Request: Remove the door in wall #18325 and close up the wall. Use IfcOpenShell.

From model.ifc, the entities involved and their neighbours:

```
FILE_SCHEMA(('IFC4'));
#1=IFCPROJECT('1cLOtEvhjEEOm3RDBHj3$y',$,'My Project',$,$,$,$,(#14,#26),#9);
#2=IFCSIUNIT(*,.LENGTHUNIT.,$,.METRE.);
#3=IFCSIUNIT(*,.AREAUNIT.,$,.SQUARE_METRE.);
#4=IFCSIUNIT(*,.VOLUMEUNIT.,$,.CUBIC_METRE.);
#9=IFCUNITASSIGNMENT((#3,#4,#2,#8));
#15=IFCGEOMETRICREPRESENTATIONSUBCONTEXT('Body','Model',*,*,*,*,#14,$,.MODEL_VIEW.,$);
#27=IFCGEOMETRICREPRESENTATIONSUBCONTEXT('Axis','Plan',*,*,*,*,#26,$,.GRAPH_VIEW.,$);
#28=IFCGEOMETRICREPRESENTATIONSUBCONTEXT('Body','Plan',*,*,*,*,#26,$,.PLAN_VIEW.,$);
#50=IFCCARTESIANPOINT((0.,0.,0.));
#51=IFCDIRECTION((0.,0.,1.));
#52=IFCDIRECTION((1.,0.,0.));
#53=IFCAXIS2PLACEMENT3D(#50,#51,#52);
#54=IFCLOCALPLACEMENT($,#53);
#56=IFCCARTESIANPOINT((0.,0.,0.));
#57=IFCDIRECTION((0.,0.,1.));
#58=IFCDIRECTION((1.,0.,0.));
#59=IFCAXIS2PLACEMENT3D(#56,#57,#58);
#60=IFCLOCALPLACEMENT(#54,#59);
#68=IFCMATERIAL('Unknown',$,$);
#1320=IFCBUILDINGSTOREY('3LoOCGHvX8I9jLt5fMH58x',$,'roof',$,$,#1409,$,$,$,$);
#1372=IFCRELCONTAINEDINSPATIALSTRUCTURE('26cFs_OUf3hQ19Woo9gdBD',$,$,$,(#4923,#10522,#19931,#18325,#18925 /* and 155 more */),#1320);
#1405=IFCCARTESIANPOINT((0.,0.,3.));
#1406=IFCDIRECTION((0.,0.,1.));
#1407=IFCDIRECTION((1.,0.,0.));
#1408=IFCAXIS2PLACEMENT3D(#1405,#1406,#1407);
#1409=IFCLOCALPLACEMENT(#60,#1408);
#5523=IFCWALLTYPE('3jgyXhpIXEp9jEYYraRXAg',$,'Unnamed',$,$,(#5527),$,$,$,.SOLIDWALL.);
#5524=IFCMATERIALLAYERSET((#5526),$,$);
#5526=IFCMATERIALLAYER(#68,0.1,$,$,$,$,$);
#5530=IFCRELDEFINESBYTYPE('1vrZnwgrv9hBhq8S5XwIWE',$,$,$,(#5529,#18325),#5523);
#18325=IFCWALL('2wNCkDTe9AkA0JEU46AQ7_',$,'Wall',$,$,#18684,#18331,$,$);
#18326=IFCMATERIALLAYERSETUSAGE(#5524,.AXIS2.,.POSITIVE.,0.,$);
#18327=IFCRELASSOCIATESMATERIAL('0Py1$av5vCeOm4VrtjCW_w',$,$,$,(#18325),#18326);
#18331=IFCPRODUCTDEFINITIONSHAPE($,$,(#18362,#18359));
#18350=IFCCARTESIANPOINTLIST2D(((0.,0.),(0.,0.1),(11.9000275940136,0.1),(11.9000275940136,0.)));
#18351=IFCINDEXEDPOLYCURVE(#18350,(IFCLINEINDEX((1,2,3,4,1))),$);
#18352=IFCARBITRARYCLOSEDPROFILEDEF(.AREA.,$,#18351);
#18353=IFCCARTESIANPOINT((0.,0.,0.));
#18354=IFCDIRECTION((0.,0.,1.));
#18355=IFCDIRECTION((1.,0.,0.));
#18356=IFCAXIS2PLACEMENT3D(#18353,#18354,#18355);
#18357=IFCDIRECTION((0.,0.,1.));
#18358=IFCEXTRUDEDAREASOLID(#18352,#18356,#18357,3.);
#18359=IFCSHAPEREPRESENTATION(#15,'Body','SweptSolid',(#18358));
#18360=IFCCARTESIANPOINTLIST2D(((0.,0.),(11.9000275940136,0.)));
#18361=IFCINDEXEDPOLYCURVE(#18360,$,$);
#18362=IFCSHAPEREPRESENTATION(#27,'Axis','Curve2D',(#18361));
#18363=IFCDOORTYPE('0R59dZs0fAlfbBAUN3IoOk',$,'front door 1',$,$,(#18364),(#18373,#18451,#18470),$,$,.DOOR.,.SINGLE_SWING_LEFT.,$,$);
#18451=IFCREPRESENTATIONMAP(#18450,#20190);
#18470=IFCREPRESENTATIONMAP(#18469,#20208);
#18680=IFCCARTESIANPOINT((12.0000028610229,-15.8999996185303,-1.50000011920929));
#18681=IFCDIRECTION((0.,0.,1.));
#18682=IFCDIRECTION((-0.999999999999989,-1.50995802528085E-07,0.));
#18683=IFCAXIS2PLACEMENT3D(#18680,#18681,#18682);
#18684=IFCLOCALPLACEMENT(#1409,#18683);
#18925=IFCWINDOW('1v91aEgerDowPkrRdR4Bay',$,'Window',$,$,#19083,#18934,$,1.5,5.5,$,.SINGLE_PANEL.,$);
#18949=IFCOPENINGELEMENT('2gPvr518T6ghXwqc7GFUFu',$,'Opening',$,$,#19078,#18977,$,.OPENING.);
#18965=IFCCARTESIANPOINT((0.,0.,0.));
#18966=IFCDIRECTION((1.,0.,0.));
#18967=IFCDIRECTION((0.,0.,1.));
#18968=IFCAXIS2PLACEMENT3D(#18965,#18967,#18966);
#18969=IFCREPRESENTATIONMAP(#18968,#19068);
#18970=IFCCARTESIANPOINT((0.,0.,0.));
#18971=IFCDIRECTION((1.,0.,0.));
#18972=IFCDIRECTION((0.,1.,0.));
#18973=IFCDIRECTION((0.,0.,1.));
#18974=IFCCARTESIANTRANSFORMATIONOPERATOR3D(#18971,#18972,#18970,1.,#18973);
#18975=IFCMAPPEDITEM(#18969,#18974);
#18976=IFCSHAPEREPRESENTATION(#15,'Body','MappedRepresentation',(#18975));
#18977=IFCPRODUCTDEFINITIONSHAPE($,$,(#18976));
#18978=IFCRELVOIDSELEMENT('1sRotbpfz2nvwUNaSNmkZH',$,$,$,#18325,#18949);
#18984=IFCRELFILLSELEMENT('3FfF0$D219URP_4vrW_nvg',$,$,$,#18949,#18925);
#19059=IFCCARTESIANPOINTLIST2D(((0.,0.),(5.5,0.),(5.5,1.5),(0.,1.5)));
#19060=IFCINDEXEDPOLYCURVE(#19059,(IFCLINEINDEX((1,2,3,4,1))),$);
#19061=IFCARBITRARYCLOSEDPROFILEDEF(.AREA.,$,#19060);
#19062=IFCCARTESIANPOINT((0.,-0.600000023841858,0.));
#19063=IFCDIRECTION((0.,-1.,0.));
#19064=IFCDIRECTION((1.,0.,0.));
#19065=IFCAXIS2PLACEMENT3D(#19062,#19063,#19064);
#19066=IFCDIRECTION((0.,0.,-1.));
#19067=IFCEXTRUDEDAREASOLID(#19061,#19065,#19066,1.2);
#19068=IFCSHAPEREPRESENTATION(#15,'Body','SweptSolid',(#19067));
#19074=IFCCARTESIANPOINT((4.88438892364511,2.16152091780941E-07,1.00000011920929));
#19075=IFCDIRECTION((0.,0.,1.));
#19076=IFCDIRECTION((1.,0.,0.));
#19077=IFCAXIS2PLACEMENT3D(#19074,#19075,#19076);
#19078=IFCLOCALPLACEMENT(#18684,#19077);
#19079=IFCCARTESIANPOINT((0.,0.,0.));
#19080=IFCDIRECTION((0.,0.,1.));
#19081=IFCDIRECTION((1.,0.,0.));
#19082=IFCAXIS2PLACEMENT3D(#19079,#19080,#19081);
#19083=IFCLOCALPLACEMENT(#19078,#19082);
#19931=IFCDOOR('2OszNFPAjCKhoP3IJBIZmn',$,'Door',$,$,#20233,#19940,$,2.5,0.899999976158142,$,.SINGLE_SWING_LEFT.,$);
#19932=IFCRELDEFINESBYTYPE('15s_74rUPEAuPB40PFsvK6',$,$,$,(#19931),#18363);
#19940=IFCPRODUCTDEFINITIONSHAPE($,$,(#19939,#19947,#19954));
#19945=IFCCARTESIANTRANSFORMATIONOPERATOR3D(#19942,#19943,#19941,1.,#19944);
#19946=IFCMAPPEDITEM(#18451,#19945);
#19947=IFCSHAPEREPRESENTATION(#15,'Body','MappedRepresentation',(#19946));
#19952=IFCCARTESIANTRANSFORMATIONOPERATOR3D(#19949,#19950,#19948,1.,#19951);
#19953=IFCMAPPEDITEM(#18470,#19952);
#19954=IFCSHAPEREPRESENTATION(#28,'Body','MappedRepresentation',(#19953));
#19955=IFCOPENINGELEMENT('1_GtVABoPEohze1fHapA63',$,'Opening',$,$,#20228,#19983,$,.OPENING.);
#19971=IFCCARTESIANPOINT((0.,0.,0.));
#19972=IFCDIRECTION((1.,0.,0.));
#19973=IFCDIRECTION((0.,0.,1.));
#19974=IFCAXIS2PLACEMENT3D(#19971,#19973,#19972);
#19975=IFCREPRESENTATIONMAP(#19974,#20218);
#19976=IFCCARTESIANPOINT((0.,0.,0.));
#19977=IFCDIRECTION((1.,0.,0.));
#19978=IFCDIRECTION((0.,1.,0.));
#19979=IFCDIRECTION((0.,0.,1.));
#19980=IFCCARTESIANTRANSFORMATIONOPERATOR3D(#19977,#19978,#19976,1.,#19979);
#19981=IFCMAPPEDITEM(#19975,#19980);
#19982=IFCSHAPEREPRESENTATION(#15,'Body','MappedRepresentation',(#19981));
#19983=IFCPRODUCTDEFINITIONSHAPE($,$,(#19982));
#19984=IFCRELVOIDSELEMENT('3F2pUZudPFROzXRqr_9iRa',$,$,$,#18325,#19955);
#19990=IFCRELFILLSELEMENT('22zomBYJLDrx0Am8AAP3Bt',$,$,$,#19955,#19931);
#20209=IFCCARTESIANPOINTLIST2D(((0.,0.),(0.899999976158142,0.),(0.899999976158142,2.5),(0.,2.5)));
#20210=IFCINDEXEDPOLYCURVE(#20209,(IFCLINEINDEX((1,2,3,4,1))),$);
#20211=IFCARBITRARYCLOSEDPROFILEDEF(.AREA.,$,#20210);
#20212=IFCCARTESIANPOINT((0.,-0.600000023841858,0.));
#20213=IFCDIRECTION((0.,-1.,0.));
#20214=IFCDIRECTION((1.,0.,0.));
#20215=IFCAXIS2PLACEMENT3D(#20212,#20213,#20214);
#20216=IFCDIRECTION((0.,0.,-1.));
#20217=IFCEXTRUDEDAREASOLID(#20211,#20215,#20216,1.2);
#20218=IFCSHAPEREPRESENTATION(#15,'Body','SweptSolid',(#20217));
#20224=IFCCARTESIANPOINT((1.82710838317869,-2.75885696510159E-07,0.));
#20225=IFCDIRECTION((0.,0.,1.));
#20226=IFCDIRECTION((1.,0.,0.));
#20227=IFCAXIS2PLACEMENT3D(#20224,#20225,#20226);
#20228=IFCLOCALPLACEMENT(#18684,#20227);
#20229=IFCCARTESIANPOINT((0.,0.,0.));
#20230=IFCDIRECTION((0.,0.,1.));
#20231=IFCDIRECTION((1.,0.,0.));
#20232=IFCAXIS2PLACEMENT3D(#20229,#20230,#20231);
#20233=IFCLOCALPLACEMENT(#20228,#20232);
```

```python
import ifcopenshell
import ifcopenshell.api.feature
import ifcopenshell.api.root
import ifcopenshell.geom
import ifcopenshell.util.shape

model = ifcopenshell.open("model.ifc")
settings = ifcopenshell.geom.settings()


def volume(element):
    """Net volume in cubic metres, openings subtracted."""
    shape = ifcopenshell.geom.create_shape(settings, element)
    return ifcopenshell.util.shape.get_volume(shape.geometry)


door = model.by_guid("2OszNFPAjCKhoP3IJBIZmn")
opening = door.FillsVoids[0].RelatingOpeningElement
wall = opening.VoidsElements[0].RelatingBuildingElement
before = volume(wall)

ifcopenshell.api.root.remove_product(model, product=door)
ifcopenshell.api.feature.remove_feature(model, feature=opening)

after = volume(wall)

print(f"wall volume {before:.3f} -> {after:.3f} m3")

model.write("model_edited.ifc")
```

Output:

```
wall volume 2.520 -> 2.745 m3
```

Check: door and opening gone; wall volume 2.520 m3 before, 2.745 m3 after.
